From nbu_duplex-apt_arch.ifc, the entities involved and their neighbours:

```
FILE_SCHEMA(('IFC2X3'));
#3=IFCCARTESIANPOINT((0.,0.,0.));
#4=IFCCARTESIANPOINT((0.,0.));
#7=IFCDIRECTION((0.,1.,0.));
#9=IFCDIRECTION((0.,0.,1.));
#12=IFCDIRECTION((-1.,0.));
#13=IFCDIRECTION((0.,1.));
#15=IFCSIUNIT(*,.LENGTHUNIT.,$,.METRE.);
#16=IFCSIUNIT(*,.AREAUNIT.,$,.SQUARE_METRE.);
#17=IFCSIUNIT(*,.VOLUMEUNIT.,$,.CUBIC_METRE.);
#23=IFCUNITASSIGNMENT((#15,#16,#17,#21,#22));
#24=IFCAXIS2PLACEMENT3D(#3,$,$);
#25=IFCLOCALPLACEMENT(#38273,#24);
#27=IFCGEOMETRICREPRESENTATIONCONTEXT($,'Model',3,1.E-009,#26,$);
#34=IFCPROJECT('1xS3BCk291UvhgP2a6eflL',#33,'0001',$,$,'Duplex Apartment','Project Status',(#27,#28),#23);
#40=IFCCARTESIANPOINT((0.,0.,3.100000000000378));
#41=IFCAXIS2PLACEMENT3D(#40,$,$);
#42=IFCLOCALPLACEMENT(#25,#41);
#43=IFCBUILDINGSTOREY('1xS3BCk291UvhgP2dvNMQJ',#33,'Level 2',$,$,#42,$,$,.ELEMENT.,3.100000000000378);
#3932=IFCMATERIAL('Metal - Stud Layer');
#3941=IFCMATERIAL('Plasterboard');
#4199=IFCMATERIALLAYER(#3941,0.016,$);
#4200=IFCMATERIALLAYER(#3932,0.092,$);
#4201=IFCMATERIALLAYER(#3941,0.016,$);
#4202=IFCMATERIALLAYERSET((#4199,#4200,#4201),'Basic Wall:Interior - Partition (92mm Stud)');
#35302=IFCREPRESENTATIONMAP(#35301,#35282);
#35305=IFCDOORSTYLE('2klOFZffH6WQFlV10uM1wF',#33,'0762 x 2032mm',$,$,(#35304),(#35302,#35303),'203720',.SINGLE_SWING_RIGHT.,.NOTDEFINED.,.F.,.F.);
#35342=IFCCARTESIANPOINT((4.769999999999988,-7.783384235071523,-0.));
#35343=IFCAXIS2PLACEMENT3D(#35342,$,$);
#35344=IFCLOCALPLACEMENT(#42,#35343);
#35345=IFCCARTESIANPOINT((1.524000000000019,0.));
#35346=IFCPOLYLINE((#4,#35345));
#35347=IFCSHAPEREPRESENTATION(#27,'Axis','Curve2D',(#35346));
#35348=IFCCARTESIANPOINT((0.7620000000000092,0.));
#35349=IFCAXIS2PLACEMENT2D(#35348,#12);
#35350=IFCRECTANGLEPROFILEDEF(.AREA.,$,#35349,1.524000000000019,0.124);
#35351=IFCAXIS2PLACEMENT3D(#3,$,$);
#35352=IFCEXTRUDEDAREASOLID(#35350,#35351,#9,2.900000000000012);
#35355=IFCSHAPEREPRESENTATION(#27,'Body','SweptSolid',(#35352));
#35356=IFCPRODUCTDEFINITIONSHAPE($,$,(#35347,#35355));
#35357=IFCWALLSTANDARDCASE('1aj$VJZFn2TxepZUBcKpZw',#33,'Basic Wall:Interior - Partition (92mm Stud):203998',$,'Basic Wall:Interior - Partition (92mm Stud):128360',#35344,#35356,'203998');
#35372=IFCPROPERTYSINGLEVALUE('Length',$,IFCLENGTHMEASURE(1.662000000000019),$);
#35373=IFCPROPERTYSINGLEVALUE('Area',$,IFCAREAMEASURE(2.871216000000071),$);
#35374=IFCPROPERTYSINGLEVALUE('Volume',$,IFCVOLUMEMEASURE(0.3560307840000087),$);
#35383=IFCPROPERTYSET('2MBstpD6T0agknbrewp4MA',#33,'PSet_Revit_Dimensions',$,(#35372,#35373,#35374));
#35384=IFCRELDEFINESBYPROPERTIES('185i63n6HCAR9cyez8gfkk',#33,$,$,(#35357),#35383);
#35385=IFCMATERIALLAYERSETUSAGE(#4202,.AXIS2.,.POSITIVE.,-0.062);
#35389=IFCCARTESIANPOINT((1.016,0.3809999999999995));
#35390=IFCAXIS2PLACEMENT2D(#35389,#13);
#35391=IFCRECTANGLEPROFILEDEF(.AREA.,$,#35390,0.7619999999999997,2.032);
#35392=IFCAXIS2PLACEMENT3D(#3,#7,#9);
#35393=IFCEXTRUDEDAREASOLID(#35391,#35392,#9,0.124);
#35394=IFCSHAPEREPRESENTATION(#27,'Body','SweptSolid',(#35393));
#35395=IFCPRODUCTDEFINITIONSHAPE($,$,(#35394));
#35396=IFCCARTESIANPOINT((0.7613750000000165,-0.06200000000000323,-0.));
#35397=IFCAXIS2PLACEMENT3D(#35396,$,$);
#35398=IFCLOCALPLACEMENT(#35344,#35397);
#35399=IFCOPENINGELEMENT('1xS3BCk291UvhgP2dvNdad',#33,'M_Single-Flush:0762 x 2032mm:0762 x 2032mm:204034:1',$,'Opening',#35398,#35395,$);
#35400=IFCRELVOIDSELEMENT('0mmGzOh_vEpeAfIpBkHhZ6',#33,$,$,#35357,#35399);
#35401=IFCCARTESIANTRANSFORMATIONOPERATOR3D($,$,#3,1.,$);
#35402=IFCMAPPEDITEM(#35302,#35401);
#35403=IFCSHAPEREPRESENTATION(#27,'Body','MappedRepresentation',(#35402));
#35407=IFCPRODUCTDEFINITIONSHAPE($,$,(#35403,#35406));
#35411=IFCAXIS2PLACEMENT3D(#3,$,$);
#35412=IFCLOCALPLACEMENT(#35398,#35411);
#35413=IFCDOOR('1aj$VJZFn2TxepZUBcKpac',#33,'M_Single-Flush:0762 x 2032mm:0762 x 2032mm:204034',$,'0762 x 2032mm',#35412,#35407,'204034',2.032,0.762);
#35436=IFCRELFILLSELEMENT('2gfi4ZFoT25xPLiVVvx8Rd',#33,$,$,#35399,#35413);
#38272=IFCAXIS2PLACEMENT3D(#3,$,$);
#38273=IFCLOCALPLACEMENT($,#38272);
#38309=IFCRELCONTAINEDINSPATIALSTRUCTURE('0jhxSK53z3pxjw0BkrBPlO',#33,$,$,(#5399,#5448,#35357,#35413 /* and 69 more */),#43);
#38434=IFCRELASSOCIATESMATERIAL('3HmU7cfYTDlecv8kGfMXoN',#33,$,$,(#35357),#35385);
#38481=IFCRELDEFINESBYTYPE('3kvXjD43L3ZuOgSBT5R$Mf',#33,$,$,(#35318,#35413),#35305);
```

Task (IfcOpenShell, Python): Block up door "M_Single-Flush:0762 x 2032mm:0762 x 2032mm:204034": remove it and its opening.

```python
import ifcopenshell
import ifcopenshell.api.feature
import ifcopenshell.api.pset
import ifcopenshell.api.root
import ifcopenshell.geom
import ifcopenshell.util.element
import ifcopenshell.util.shape
import ifcopenshell.util.unit

model = ifcopenshell.open("nbu_duplex-apt_arch.ifc")
area_scale = ifcopenshell.util.unit.calculate_unit_scale(model, "AREAUNIT")
volume_scale = ifcopenshell.util.unit.calculate_unit_scale(model, "VOLUMEUNIT")
settings = ifcopenshell.geom.settings()


def volume(element):
    """Net volume in cubic metres, openings subtracted."""
    shape = ifcopenshell.geom.create_shape(settings, element)
    return ifcopenshell.util.shape.get_volume(shape.geometry)


door = model.by_guid("1aj$VJZFn2TxepZUBcKpac")
opening = door.FillsVoids[0].RelatingOpeningElement
wall = opening.VoidsElements[0].RelatingBuildingElement
before = volume(wall)

ifcopenshell.api.root.remove_product(model, product=door)
ifcopenshell.api.feature.remove_feature(model, feature=opening)

after = volume(wall)
thickness = 0.124  # wall thickness in metres

# Update the wall's stored quantities.
pset = model.by_id(ifcopenshell.util.element.get_pset(wall, "PSet_Revit_Dimensions", should_inherit=False)["id"])
ifcopenshell.api.pset.edit_pset(model, pset=pset, properties={
    "Area": model.create_entity("IfcAreaMeasure", after / thickness / area_scale),
    "Volume": model.create_entity("IfcVolumeMeasure", after / volume_scale),
})

print(f"wall volume {before:.3f} -> {after:.3f} m3")

model.write("nbu_duplex-apt_arch_updated.ifc")
```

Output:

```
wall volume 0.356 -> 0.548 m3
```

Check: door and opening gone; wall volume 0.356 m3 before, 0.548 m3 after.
